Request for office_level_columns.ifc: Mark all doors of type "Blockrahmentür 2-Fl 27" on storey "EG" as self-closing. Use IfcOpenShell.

First a look at what the model holds.

```python
import ifcopenshell
import ifcopenshell.util.element

model = ifcopenshell.open("office_level_columns.ifc")
print(model.schema)
storey = next(s for s in model.by_type("IfcBuildingStorey") if s.Name == "EG")
doors = [e for e in ifcopenshell.util.element.get_decomposition(storey) if e.is_a("IfcDoor")]
seen = {}
for e in doors:
    element_type = ifcopenshell.util.element.get_type(e)
    key = (element_type.Name if element_type != e and element_type else None, ifcopenshell.util.element.get_pset(e, "Pset_DoorCommon", "SelfClosing"))
    seen[key] = seen.get(key, 0) + 1
for (name, value), count in sorted(seen.items(), key=str):
    print(count, "x", name, "|", value)
```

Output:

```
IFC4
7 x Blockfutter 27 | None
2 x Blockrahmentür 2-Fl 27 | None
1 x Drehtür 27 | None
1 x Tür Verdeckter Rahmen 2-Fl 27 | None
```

```python
import ifcopenshell
import ifcopenshell.api.pset
import ifcopenshell.util.element

model = ifcopenshell.open("office_level_columns.ifc")

storey = next(s for s in model.by_type("IfcBuildingStorey") if s.Name == "EG")
doors = [e for e in ifcopenshell.util.element.get_decomposition(storey) if e.is_a("IfcDoor")]

count = 0
for e in doors:
    element_type = ifcopenshell.util.element.get_type(e)
    if element_type in (None, e) or element_type.Name != "Blockrahmentür 2-Fl 27":
        continue
    # add_pset returns the element's existing set when there is one.
    pset = ifcopenshell.api.pset.add_pset(model, product=e, name="Pset_DoorCommon")
    ifcopenshell.api.pset.edit_pset(model, pset=pset, properties={"SelfClosing": True})
    count += 1

print(count, "doors updated")

model.write("office_level_columns_rev.ifc")
```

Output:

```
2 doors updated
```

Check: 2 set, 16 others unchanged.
